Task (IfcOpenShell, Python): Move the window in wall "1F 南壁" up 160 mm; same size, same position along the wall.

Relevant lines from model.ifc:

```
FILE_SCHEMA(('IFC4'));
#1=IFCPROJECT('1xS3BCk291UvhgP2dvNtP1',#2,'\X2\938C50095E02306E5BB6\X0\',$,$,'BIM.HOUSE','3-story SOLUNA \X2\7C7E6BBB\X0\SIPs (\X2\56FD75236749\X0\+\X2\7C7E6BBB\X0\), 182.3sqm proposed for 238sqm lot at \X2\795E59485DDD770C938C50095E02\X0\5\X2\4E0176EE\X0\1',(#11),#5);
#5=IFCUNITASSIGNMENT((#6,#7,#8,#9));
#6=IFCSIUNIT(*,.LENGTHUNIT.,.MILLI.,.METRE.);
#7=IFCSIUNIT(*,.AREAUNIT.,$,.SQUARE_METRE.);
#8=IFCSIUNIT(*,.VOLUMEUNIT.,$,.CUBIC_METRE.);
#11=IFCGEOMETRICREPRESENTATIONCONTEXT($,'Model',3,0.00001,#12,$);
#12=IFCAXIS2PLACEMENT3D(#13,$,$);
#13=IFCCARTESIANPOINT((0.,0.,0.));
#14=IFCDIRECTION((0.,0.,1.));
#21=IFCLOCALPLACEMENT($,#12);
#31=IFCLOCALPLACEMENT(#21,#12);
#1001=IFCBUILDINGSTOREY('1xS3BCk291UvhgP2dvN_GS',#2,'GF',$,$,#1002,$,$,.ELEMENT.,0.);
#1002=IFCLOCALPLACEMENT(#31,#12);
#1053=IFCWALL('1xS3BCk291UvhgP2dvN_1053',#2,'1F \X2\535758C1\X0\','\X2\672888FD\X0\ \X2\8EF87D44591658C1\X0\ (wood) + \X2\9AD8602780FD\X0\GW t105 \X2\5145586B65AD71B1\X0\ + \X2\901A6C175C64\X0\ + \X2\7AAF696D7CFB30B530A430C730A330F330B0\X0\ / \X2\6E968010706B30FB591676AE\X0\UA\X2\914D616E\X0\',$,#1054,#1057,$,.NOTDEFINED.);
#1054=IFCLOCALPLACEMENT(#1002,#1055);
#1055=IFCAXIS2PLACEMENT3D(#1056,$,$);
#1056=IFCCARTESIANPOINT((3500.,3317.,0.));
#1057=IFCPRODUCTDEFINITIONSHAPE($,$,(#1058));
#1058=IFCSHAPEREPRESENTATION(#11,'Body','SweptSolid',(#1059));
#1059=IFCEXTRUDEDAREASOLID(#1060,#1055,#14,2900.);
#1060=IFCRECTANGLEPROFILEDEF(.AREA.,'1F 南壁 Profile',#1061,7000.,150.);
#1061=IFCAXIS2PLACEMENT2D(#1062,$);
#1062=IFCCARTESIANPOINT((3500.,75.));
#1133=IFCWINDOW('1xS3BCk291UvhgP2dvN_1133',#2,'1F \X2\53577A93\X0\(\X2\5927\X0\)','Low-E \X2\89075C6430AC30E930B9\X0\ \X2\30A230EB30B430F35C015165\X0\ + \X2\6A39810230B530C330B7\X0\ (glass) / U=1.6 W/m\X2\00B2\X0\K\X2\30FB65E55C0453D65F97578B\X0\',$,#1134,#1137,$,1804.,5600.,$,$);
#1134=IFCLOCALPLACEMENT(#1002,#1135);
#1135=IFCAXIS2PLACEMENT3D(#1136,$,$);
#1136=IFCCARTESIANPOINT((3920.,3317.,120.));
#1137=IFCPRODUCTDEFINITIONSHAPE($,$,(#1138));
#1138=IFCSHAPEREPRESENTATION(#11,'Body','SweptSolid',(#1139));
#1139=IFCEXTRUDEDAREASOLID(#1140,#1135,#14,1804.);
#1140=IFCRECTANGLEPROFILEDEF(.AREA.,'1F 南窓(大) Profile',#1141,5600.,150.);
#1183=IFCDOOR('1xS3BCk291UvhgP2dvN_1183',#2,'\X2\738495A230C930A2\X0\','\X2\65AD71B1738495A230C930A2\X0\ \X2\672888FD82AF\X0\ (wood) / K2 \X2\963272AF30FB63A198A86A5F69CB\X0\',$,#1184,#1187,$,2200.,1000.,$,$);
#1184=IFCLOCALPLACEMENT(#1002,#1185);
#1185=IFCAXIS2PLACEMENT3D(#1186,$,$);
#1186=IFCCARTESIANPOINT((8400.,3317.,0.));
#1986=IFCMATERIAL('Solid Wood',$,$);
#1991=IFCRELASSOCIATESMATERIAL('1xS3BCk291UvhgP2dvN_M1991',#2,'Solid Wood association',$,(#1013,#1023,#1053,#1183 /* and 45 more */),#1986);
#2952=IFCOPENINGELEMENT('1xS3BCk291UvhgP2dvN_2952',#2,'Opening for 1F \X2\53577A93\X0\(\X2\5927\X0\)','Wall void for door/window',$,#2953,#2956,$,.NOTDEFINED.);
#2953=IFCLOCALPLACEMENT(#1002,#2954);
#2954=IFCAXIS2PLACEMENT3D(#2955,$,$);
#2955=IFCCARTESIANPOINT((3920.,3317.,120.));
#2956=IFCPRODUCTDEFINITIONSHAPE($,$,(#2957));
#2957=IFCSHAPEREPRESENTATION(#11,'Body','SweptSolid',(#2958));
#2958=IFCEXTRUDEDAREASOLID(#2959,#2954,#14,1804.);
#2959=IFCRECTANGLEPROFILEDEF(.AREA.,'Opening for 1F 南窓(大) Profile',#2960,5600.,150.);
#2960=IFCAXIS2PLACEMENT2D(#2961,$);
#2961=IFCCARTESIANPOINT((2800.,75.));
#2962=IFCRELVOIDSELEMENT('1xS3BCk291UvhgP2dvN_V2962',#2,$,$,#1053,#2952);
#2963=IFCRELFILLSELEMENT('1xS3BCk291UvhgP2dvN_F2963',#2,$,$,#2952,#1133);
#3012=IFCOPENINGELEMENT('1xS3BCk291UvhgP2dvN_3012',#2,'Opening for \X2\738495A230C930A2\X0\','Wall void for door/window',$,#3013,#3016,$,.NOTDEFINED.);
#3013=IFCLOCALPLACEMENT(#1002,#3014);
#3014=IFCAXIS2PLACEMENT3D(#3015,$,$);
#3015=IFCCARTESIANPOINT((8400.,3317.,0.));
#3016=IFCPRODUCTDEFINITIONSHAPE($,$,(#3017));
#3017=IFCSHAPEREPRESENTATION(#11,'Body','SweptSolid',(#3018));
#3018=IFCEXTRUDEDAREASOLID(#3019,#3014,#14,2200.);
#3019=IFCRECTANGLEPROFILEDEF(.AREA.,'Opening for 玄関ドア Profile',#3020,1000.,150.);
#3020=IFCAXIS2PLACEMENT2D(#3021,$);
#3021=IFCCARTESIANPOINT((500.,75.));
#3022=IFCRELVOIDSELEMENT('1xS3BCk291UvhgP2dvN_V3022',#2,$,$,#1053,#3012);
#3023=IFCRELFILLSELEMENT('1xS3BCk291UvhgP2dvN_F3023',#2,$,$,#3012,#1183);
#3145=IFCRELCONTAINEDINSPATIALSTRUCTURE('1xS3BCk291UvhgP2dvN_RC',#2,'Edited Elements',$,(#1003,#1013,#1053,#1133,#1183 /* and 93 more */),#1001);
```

```python
import numpy as np
import ifcopenshell
import ifcopenshell.api.geometry
import ifcopenshell.util.placement
import ifcopenshell.util.unit

model = ifcopenshell.open("model.ifc")
unit_scale = ifcopenshell.util.unit.calculate_unit_scale(model)

window = model.by_guid("1xS3BCk291UvhgP2dvN_1133")
opening = window.FillsVoids[0].RelatingOpeningElement
dz = 160.0

shift = np.array([0.0, 0.0, dz])
# The window is not placed relative to its opening, so move both.
for product in (opening, window):
    matrix = ifcopenshell.util.placement.get_local_placement(product.ObjectPlacement)
    matrix[:3, 3] += shift
    ifcopenshell.api.geometry.edit_object_placement(model, product=product, matrix=matrix, is_si=False)

print(f"moved by {dz * unit_scale:+.3f} m")

model.write("model_updated.ifc")
```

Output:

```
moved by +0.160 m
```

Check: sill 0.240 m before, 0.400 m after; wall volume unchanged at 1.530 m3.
